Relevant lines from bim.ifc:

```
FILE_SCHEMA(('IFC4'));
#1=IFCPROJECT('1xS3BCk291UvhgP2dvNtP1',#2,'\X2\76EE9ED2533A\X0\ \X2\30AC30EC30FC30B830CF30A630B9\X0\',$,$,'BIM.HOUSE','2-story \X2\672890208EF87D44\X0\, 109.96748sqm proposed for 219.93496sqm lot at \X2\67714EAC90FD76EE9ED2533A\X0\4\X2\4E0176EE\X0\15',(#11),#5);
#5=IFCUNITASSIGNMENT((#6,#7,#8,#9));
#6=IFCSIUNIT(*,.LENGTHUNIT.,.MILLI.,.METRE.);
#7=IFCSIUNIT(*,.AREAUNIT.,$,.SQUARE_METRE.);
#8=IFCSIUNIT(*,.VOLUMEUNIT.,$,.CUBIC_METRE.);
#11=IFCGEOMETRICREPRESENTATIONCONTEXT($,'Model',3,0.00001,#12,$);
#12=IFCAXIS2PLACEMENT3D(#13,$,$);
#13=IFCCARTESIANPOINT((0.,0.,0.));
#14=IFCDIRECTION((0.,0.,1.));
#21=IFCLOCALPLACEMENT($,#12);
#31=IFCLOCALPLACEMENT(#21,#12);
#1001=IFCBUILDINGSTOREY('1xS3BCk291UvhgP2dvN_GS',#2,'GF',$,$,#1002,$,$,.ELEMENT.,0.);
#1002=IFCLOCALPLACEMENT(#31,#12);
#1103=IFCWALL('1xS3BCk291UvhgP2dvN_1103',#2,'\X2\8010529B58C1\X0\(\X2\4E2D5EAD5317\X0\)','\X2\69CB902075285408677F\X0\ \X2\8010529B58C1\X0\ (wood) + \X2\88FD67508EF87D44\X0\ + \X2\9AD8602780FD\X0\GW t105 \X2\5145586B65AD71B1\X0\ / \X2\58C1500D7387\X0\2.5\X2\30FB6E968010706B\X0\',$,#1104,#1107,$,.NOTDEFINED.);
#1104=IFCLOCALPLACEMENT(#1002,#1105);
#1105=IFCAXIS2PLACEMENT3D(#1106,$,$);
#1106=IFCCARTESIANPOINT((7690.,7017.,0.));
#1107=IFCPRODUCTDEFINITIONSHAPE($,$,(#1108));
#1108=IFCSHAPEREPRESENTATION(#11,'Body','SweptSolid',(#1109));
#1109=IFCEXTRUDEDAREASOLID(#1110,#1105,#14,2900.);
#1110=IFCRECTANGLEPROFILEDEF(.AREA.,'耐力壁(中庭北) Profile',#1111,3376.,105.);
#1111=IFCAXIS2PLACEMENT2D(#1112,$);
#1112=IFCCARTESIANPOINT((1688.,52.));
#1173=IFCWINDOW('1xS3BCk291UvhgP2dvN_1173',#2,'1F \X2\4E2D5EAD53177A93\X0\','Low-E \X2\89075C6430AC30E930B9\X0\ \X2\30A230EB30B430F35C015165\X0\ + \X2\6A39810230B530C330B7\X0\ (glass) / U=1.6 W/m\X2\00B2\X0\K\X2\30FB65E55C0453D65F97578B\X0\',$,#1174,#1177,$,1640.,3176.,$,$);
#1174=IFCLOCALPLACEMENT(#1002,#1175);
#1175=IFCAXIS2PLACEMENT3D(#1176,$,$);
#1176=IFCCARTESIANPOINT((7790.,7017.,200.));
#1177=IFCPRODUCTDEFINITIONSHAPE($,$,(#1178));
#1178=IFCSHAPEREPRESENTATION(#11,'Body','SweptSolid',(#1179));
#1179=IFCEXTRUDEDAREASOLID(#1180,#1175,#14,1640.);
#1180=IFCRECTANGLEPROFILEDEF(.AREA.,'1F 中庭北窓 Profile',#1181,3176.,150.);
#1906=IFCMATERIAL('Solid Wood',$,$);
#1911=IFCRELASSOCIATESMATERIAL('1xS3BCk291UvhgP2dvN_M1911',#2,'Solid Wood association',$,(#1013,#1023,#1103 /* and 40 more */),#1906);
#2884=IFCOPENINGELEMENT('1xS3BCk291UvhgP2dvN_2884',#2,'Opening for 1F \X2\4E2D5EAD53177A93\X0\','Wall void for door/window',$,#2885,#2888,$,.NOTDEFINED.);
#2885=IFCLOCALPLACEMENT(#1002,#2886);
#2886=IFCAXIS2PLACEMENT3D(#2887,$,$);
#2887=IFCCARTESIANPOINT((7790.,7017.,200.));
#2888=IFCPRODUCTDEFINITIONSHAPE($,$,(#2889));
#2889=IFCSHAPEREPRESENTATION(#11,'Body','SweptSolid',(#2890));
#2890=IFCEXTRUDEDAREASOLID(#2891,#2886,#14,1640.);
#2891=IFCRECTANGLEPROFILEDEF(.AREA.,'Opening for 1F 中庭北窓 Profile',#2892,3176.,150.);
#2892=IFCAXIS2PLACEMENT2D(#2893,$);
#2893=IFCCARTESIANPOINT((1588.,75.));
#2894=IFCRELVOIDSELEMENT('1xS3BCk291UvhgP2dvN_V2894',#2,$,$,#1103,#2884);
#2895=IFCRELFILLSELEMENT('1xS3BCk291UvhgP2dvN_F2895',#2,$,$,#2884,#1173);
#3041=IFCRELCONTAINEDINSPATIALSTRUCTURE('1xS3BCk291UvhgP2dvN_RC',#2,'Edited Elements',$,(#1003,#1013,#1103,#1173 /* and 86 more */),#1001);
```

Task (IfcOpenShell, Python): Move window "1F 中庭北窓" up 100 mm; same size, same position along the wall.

```python
import numpy as np
import ifcopenshell
import ifcopenshell.api.geometry
import ifcopenshell.util.placement
import ifcopenshell.util.unit

model = ifcopenshell.open("bim.ifc")
unit_scale = ifcopenshell.util.unit.calculate_unit_scale(model)

window = model.by_guid("1xS3BCk291UvhgP2dvN_1173")
opening = window.FillsVoids[0].RelatingOpeningElement
dz = 0.1 / unit_scale

shift = np.array([0.0, 0.0, dz])
# The window is not placed relative to its opening, so move both.
for product in (opening, window):
    matrix = ifcopenshell.util.placement.get_local_placement(product.ObjectPlacement)
    matrix[:3, 3] += shift
    ifcopenshell.api.geometry.edit_object_placement(model, product=product, matrix=matrix, is_si=False)

print(f"moved by {dz * unit_scale:+.3f} m")

model.write("bim_v2.ifc")
```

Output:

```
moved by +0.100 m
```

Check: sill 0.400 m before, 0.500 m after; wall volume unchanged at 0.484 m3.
